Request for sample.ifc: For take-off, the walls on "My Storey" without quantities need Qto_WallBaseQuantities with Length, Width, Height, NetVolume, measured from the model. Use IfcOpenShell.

First a look at what the model holds.

```python
import ifcopenshell
import ifcopenshell.util.element
import ifcopenshell.util.unit

model = ifcopenshell.open("sample.ifc")
print(model.schema)
for unit_type in ("LENGTHUNIT", "AREAUNIT", "VOLUMEUNIT"):
    print(unit_type, ifcopenshell.util.unit.calculate_unit_scale(model, unit_type))
storey = next(s for s in model.by_type("IfcBuildingStorey") if s.Name == "My Storey")
walls = [e for e in ifcopenshell.util.element.get_decomposition(storey) if e.is_a("IfcWall")]
for e in sorted(walls, key=lambda e: e.id()):
    print(e.id(), e.is_a(), e.Name, list(ifcopenshell.util.element.get_psets(e, qtos_only=True)), sep=" | ")
```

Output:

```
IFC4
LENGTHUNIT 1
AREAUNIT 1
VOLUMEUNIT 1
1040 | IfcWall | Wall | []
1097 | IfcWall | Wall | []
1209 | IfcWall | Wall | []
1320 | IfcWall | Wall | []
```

```python
import ifcopenshell
import ifcopenshell.api.pset
import ifcopenshell.geom
import ifcopenshell.util.element
import ifcopenshell.util.shape
import ifcopenshell.util.unit

model = ifcopenshell.open("sample.ifc")
unit_scale = ifcopenshell.util.unit.calculate_unit_scale(model)
volume_scale = ifcopenshell.util.unit.calculate_unit_scale(model, "VOLUMEUNIT")
settings = ifcopenshell.geom.settings()

storey = next(s for s in model.by_type("IfcBuildingStorey") if s.Name == "My Storey")
walls = [e for e in ifcopenshell.util.element.get_decomposition(storey) if e.is_a("IfcWall")]

for e in sorted(walls, key=lambda e: e.id()):
    if ifcopenshell.util.element.get_psets(e, qtos_only=True, should_inherit=False):
        continue
    # Geometry comes back in metres, in the element's own axes.
    shape = ifcopenshell.geom.create_shape(settings, e)
    values = {
        "Length": ifcopenshell.util.shape.get_x(shape.geometry) / unit_scale,
        "Width": ifcopenshell.util.shape.get_y(shape.geometry) / unit_scale,
        "Height": ifcopenshell.util.shape.get_z(shape.geometry) / unit_scale,
        "NetVolume": ifcopenshell.util.shape.get_volume(shape.geometry) / volume_scale,
    }
    qto = ifcopenshell.api.pset.add_qto(model, product=e, name="Qto_WallBaseQuantities")
    ifcopenshell.api.pset.edit_qto(model, qto=qto, properties=values)
    print(e.id(), {k: round(v, 3) for k, v in values.items()})

model.write("sample_edited.ifc")
```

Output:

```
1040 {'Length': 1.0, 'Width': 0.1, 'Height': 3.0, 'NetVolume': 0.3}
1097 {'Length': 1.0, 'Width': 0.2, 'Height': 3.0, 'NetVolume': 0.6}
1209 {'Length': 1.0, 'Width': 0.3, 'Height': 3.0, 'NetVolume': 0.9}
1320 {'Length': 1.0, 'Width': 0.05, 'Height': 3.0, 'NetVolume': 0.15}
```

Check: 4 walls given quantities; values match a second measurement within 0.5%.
